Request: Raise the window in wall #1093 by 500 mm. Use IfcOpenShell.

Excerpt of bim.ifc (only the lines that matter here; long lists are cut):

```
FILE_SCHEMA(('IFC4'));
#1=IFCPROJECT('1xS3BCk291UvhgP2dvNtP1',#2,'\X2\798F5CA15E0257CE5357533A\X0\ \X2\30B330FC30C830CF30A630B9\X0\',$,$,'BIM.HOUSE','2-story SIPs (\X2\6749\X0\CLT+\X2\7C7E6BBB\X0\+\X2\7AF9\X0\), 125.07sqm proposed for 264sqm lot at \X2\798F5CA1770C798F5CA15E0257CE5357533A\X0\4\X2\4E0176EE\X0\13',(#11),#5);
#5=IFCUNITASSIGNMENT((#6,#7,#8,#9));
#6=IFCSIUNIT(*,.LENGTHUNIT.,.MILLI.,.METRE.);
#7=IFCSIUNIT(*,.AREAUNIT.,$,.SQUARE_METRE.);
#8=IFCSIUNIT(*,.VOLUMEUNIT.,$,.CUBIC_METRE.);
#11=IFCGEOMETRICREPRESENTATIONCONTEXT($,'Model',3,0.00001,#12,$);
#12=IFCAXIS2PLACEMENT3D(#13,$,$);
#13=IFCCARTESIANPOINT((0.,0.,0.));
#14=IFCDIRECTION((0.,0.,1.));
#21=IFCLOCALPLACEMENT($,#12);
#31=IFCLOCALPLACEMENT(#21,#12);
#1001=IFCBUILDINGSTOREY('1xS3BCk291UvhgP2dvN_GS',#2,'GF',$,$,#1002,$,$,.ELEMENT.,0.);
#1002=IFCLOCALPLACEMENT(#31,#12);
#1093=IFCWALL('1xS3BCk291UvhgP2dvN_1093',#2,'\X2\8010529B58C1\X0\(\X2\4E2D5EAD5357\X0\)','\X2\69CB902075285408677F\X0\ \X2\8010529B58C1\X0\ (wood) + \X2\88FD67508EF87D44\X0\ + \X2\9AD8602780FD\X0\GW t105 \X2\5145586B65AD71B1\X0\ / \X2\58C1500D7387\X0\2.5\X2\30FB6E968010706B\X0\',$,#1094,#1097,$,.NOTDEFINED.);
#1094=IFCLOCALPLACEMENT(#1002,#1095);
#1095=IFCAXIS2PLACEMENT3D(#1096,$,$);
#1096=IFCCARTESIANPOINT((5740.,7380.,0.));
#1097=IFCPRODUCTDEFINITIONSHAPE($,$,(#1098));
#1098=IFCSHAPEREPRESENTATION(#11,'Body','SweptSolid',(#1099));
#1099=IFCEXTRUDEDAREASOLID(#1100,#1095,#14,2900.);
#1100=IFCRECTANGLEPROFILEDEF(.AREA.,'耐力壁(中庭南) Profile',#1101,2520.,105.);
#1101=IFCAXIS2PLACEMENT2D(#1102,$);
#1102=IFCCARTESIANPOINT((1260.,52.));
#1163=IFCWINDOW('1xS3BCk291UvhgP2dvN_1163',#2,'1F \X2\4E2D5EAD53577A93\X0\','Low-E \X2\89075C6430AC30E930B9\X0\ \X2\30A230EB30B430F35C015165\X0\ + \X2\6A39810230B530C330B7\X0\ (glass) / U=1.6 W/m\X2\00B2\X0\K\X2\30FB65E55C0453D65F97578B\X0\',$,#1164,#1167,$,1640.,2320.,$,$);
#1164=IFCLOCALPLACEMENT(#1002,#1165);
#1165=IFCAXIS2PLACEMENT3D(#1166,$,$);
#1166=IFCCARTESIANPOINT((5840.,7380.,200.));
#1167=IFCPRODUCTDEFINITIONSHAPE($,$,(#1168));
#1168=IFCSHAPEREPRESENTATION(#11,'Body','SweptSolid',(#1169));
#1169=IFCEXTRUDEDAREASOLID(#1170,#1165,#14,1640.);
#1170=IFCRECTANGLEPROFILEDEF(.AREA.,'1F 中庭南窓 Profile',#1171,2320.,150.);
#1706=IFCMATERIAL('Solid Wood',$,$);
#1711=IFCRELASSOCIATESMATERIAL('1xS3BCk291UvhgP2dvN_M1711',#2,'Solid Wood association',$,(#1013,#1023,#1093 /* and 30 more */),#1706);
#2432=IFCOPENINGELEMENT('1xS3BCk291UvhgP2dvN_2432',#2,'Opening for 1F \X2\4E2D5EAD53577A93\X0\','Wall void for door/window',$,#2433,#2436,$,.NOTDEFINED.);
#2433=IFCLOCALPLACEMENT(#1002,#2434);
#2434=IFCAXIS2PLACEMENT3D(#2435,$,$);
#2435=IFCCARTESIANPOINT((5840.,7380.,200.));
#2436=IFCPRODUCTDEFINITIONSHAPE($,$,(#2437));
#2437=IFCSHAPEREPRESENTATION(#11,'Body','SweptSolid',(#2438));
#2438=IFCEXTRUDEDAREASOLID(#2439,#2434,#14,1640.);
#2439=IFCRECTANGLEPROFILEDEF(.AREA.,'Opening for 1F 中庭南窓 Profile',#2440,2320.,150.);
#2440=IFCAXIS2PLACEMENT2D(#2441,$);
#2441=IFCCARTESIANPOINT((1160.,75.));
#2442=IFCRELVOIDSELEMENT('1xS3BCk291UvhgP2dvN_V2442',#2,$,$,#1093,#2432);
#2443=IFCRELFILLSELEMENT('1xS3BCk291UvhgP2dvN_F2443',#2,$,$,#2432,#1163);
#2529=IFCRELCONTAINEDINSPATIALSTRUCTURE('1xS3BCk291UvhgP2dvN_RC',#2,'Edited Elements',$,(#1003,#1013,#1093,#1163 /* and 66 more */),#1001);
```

```python
import numpy as np
import ifcopenshell
import ifcopenshell.api.geometry
import ifcopenshell.util.placement
import ifcopenshell.util.unit

model = ifcopenshell.open("bim.ifc")
unit_scale = ifcopenshell.util.unit.calculate_unit_scale(model)

window = model.by_guid("1xS3BCk291UvhgP2dvN_1163")
opening = window.FillsVoids[0].RelatingOpeningElement
dz = 0.5 / unit_scale

shift = np.array([0.0, 0.0, dz])
# The window is not placed relative to its opening, so move both.
for product in (opening, window):
    matrix = ifcopenshell.util.placement.get_local_placement(product.ObjectPlacement)
    matrix[:3, 3] += shift
    ifcopenshell.api.geometry.edit_object_placement(model, product=product, matrix=matrix, is_si=False)

print(f"moved by {dz * unit_scale:+.3f} m")

model.write("bim_updated.ifc")
```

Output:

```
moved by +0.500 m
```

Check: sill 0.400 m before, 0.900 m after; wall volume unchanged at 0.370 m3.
